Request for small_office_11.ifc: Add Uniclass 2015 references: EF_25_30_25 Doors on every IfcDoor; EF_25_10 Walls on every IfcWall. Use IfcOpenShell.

First a look at what the model holds.

```python
import ifcopenshell

model = ifcopenshell.open("small_office_11.ifc")
print(model.schema)
print("classifications:", [c.Name for c in model.by_type("IfcClassification")])
for ifc_class in ("IfcDoor", "IfcRoof", "IfcStair", "IfcWall", "IfcWindow"):
    print(ifc_class, len(model.by_type(ifc_class)))
```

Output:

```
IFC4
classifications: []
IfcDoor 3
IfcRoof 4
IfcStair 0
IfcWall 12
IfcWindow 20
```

```python
import ifcopenshell
import ifcopenshell.api.classification

model = ifcopenshell.open("small_office_11.ifc")

system = ifcopenshell.api.classification.add_classification(model, classification="Uniclass 2015")

codes = {
    "IfcDoor": ("EF_25_30_25", "Doors"),
    "IfcWall": ("EF_25_10", "Walls"),
}
for ifc_class, (code, name) in codes.items():
    products = model.by_type(ifc_class)
    ifcopenshell.api.classification.add_reference(
        model, products=products, classification=system, identification=code, name=name
    )
    print(code, len(products))

model.write("small_office_11_v2.ifc")
```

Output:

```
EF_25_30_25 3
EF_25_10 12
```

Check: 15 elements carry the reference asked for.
